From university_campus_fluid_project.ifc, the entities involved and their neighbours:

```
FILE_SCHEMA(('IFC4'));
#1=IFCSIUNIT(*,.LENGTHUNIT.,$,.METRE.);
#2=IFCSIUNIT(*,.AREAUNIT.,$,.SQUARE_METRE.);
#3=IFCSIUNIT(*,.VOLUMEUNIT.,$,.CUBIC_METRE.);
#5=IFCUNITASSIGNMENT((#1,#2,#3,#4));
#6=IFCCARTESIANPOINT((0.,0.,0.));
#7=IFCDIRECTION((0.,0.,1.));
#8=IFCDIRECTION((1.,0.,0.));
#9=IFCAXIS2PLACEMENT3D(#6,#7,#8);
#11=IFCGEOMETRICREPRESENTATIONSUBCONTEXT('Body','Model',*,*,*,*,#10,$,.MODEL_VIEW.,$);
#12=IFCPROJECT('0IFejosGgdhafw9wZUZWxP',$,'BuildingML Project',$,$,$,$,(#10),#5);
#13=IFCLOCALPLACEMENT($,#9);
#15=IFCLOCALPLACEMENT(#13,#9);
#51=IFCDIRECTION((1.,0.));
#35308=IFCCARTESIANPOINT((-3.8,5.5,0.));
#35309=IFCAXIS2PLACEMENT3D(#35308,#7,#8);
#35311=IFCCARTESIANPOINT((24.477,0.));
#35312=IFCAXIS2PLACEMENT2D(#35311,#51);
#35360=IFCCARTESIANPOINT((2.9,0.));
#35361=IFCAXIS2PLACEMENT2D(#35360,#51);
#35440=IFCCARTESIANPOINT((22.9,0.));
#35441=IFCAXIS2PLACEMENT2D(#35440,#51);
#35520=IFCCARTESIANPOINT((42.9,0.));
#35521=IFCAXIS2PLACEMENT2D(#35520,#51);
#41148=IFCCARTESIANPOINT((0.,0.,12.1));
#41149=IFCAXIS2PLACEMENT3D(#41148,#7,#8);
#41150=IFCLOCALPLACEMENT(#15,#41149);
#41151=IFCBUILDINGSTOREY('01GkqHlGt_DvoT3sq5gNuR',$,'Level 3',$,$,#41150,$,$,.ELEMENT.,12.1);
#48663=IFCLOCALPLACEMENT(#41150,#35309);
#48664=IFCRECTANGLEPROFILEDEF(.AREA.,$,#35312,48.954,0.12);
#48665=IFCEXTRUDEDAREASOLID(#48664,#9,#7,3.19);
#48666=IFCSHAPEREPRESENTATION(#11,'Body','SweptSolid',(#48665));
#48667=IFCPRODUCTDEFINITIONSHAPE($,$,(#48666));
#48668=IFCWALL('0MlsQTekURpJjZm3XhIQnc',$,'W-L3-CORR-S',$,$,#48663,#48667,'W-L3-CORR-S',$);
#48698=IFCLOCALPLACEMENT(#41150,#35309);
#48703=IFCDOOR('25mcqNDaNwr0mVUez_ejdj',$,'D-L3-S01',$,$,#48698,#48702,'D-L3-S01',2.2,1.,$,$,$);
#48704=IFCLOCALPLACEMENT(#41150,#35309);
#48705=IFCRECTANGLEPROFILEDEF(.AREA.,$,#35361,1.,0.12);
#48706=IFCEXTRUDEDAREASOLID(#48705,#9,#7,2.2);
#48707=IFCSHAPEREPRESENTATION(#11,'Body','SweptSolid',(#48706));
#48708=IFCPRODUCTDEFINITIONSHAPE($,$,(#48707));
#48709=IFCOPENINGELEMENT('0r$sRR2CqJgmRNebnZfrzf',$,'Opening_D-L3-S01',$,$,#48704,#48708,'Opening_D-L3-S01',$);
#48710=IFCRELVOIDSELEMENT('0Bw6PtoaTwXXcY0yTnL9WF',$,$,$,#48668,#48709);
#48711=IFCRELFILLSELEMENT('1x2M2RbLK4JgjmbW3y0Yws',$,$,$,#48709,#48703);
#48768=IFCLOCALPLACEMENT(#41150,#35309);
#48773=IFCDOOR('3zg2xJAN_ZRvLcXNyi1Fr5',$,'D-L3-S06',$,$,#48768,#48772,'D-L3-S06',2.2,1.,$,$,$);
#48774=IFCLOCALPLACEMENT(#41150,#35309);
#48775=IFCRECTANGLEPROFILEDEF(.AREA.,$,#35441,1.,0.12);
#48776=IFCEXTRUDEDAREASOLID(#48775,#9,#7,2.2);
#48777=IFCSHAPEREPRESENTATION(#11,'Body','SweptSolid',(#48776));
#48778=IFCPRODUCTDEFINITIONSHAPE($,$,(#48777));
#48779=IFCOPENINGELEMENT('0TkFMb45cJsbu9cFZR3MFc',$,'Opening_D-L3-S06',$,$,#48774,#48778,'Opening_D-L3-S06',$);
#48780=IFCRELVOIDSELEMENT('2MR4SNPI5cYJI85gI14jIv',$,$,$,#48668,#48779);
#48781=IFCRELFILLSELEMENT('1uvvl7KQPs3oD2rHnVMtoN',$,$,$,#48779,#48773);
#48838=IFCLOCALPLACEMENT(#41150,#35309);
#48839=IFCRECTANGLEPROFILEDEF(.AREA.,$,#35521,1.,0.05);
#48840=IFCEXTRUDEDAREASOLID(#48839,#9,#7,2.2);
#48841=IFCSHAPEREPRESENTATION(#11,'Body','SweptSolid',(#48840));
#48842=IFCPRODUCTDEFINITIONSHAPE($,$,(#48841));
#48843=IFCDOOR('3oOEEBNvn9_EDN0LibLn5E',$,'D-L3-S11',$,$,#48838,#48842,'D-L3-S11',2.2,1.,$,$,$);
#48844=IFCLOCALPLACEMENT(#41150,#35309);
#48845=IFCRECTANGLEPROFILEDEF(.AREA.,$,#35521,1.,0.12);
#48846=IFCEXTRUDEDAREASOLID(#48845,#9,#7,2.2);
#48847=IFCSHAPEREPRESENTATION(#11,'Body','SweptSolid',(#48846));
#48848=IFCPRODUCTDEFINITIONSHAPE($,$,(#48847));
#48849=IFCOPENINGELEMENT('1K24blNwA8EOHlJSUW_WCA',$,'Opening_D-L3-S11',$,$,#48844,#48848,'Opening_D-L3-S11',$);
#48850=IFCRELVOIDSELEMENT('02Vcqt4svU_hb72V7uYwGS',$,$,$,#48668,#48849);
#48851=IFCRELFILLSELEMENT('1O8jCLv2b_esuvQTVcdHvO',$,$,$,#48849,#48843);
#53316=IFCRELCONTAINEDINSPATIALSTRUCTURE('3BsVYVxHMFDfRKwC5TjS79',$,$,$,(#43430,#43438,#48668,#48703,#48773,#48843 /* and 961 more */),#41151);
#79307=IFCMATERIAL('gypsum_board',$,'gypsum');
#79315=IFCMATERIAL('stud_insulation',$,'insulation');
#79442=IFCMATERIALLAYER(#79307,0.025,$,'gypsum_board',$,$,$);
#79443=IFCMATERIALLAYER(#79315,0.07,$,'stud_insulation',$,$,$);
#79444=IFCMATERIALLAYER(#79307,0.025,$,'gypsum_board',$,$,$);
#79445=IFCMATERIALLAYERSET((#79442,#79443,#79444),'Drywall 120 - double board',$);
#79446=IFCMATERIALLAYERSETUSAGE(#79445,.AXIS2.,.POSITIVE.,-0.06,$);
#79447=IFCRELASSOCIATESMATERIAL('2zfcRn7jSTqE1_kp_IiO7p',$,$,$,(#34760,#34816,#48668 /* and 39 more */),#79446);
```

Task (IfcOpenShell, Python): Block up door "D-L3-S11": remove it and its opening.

```python
import ifcopenshell
import ifcopenshell.api.feature
import ifcopenshell.api.root
import ifcopenshell.geom
import ifcopenshell.util.shape

model = ifcopenshell.open("university_campus_fluid_project.ifc")
settings = ifcopenshell.geom.settings()


def volume(element):
    """Net volume in cubic metres, openings subtracted."""
    shape = ifcopenshell.geom.create_shape(settings, element)
    return ifcopenshell.util.shape.get_volume(shape.geometry)


door = model.by_guid("3oOEEBNvn9_EDN0LibLn5E")
opening = door.FillsVoids[0].RelatingOpeningElement
wall = opening.VoidsElements[0].RelatingBuildingElement
before = volume(wall)

ifcopenshell.api.root.remove_product(model, product=door)
ifcopenshell.api.feature.remove_feature(model, feature=opening)

after = volume(wall)

print(f"wall volume {before:.3f} -> {after:.3f} m3")

model.write("university_campus_fluid_project_updated.ifc")
```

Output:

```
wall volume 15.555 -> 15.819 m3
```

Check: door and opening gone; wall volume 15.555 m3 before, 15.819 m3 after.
